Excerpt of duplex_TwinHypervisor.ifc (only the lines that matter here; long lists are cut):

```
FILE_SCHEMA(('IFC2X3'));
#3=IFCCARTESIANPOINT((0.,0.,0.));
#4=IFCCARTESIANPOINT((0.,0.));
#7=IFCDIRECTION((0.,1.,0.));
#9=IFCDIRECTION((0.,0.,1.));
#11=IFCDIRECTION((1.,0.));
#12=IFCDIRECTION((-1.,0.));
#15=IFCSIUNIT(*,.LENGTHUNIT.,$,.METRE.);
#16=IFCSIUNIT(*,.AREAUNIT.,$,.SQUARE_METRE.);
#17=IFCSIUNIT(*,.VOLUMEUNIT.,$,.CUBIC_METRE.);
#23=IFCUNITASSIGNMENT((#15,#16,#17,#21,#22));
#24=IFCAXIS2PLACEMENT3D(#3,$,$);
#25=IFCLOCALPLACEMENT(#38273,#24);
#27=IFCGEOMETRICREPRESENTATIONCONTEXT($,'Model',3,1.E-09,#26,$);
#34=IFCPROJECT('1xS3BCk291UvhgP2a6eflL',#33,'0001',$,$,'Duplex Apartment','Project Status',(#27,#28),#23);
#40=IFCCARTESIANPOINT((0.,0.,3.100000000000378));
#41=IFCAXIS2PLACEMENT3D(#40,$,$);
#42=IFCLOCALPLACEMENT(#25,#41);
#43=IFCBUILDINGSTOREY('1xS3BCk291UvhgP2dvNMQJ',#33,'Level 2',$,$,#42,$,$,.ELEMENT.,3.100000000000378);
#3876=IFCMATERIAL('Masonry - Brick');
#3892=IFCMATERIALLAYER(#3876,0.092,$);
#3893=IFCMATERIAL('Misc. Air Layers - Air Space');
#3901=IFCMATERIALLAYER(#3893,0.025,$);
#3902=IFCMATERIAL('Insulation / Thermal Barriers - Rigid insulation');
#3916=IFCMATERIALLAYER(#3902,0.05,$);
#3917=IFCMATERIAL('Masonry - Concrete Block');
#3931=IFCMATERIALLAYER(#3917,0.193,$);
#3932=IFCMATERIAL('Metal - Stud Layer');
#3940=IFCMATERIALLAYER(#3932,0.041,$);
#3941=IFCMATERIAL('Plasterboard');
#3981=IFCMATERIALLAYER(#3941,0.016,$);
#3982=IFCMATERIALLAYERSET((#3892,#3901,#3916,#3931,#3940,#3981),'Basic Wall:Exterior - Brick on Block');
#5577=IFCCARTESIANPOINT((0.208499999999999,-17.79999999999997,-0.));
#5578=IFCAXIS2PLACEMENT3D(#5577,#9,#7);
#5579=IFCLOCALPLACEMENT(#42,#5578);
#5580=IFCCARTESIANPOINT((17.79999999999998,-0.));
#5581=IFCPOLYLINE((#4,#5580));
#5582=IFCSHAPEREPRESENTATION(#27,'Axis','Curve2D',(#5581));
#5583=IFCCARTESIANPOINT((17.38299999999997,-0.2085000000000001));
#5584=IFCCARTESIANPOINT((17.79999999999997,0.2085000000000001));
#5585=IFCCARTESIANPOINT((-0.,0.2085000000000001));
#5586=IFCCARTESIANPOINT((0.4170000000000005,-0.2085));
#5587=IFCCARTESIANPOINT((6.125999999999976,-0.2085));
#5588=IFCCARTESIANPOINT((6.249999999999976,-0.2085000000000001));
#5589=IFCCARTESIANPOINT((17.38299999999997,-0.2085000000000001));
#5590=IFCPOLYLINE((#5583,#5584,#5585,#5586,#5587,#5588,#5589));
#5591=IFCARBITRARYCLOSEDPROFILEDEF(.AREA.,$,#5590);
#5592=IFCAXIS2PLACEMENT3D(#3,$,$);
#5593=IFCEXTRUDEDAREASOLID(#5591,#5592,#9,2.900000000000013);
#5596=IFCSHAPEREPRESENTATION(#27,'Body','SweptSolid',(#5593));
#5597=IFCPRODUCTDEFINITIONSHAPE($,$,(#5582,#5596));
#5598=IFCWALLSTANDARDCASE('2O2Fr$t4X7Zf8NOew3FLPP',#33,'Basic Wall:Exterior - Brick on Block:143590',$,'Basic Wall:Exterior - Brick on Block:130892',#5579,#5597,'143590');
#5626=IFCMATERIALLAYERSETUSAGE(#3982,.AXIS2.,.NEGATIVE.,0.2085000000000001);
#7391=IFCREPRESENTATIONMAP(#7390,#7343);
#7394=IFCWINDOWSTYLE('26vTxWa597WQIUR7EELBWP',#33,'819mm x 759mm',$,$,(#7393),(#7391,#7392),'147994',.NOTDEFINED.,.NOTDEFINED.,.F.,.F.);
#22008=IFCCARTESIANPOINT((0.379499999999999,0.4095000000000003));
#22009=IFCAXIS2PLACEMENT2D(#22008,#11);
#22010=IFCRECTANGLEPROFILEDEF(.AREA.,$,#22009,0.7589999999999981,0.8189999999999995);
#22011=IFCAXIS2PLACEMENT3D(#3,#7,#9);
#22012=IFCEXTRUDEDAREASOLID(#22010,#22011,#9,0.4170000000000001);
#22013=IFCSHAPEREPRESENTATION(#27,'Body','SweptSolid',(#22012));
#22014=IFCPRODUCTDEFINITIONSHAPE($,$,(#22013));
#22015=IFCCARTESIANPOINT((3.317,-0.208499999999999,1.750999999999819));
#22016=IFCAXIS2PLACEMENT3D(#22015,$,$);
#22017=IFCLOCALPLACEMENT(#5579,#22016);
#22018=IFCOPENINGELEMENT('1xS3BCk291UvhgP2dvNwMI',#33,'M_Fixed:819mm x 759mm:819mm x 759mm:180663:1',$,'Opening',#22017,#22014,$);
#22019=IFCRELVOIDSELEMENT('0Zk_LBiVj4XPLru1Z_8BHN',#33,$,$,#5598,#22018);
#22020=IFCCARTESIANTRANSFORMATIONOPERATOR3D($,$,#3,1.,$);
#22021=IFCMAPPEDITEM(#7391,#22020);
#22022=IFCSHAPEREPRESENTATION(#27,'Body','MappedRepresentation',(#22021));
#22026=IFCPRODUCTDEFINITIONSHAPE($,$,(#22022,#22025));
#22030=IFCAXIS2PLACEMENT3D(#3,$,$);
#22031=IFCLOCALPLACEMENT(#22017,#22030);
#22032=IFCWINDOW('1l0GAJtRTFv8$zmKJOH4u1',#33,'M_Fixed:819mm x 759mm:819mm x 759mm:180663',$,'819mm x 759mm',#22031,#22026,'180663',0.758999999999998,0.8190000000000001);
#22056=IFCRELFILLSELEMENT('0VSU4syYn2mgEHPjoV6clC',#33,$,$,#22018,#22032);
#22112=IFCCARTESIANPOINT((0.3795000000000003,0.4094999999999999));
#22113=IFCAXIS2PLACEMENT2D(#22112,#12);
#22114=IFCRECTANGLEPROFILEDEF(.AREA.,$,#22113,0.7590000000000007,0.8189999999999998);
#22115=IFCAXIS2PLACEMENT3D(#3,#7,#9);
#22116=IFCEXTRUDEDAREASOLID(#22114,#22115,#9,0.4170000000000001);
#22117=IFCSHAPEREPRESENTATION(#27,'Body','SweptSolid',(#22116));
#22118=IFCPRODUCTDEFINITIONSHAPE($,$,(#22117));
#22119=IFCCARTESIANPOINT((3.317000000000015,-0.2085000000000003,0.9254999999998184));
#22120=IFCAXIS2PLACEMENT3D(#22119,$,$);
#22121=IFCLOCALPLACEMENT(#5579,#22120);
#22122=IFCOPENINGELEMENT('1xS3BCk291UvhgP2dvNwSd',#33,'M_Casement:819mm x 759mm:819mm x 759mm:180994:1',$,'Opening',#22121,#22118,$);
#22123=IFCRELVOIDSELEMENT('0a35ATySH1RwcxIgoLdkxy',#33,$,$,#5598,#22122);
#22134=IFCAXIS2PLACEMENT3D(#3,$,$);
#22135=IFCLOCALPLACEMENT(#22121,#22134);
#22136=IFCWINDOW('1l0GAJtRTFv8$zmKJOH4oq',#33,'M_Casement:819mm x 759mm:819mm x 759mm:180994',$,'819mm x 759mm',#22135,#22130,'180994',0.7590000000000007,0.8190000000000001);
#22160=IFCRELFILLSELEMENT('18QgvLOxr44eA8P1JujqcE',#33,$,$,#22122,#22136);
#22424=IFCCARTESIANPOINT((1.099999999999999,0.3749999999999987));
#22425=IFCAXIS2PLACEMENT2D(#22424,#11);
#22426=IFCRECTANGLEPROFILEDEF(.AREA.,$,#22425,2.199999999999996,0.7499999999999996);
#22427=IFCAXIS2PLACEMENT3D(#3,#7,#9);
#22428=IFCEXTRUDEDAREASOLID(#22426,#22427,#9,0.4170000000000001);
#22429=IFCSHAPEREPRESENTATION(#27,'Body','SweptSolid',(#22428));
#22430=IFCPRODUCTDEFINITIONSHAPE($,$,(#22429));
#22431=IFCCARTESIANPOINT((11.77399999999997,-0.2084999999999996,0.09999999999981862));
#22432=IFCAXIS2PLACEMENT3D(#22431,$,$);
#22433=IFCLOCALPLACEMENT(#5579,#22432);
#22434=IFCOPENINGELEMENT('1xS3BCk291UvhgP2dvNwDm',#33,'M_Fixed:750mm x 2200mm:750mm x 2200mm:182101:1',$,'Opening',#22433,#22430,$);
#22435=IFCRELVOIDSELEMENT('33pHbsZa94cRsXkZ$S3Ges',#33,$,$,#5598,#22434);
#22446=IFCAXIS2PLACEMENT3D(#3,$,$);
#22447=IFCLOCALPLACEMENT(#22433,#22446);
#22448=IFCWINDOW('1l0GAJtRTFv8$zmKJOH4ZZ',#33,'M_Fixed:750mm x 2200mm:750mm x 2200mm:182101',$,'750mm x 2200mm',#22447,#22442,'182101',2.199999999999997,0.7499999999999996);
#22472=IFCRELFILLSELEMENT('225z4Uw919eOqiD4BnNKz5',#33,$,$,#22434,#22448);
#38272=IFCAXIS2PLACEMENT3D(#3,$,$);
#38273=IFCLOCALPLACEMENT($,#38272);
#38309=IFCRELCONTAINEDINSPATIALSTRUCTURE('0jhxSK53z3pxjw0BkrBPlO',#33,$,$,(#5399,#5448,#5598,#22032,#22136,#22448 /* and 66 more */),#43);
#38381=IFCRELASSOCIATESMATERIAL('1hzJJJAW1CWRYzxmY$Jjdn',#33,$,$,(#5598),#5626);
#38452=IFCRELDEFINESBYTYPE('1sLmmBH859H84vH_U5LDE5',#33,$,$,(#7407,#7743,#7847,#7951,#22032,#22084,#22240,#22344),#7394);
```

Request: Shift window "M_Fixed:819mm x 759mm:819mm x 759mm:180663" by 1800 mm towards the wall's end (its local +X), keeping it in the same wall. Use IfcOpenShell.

```python
import ifcopenshell
import ifcopenshell.api.geometry
import ifcopenshell.util.placement
import ifcopenshell.util.unit

model = ifcopenshell.open("duplex_TwinHypervisor.ifc")
unit_scale = ifcopenshell.util.unit.calculate_unit_scale(model)

window = model.by_id(22032)
opening = window.FillsVoids[0].RelatingOpeningElement
wall = opening.VoidsElements[0].RelatingBuildingElement

wall_matrix = ifcopenshell.util.placement.get_local_placement(wall.ObjectPlacement)
shift = wall_matrix[:3, 0] * 1.8 / unit_scale
before = ifcopenshell.util.placement.get_local_placement(window.ObjectPlacement)[:3, 3].copy()

# The window is placed relative to its opening, so it follows when the opening moves.
matrix = ifcopenshell.util.placement.get_local_placement(opening.ObjectPlacement)
matrix[:3, 3] += shift
ifcopenshell.api.geometry.edit_object_placement(
    model, product=opening, matrix=matrix, is_si=False, should_transform_children=True
)

after = ifcopenshell.util.placement.get_local_placement(window.ObjectPlacement)[:3, 3]
print("window moved by", (after - before).round(3) + 0.0)

model.write("duplex_TwinHypervisor_v2.ifc")
```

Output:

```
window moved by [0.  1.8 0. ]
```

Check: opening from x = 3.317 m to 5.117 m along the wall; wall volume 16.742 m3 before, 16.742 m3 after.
